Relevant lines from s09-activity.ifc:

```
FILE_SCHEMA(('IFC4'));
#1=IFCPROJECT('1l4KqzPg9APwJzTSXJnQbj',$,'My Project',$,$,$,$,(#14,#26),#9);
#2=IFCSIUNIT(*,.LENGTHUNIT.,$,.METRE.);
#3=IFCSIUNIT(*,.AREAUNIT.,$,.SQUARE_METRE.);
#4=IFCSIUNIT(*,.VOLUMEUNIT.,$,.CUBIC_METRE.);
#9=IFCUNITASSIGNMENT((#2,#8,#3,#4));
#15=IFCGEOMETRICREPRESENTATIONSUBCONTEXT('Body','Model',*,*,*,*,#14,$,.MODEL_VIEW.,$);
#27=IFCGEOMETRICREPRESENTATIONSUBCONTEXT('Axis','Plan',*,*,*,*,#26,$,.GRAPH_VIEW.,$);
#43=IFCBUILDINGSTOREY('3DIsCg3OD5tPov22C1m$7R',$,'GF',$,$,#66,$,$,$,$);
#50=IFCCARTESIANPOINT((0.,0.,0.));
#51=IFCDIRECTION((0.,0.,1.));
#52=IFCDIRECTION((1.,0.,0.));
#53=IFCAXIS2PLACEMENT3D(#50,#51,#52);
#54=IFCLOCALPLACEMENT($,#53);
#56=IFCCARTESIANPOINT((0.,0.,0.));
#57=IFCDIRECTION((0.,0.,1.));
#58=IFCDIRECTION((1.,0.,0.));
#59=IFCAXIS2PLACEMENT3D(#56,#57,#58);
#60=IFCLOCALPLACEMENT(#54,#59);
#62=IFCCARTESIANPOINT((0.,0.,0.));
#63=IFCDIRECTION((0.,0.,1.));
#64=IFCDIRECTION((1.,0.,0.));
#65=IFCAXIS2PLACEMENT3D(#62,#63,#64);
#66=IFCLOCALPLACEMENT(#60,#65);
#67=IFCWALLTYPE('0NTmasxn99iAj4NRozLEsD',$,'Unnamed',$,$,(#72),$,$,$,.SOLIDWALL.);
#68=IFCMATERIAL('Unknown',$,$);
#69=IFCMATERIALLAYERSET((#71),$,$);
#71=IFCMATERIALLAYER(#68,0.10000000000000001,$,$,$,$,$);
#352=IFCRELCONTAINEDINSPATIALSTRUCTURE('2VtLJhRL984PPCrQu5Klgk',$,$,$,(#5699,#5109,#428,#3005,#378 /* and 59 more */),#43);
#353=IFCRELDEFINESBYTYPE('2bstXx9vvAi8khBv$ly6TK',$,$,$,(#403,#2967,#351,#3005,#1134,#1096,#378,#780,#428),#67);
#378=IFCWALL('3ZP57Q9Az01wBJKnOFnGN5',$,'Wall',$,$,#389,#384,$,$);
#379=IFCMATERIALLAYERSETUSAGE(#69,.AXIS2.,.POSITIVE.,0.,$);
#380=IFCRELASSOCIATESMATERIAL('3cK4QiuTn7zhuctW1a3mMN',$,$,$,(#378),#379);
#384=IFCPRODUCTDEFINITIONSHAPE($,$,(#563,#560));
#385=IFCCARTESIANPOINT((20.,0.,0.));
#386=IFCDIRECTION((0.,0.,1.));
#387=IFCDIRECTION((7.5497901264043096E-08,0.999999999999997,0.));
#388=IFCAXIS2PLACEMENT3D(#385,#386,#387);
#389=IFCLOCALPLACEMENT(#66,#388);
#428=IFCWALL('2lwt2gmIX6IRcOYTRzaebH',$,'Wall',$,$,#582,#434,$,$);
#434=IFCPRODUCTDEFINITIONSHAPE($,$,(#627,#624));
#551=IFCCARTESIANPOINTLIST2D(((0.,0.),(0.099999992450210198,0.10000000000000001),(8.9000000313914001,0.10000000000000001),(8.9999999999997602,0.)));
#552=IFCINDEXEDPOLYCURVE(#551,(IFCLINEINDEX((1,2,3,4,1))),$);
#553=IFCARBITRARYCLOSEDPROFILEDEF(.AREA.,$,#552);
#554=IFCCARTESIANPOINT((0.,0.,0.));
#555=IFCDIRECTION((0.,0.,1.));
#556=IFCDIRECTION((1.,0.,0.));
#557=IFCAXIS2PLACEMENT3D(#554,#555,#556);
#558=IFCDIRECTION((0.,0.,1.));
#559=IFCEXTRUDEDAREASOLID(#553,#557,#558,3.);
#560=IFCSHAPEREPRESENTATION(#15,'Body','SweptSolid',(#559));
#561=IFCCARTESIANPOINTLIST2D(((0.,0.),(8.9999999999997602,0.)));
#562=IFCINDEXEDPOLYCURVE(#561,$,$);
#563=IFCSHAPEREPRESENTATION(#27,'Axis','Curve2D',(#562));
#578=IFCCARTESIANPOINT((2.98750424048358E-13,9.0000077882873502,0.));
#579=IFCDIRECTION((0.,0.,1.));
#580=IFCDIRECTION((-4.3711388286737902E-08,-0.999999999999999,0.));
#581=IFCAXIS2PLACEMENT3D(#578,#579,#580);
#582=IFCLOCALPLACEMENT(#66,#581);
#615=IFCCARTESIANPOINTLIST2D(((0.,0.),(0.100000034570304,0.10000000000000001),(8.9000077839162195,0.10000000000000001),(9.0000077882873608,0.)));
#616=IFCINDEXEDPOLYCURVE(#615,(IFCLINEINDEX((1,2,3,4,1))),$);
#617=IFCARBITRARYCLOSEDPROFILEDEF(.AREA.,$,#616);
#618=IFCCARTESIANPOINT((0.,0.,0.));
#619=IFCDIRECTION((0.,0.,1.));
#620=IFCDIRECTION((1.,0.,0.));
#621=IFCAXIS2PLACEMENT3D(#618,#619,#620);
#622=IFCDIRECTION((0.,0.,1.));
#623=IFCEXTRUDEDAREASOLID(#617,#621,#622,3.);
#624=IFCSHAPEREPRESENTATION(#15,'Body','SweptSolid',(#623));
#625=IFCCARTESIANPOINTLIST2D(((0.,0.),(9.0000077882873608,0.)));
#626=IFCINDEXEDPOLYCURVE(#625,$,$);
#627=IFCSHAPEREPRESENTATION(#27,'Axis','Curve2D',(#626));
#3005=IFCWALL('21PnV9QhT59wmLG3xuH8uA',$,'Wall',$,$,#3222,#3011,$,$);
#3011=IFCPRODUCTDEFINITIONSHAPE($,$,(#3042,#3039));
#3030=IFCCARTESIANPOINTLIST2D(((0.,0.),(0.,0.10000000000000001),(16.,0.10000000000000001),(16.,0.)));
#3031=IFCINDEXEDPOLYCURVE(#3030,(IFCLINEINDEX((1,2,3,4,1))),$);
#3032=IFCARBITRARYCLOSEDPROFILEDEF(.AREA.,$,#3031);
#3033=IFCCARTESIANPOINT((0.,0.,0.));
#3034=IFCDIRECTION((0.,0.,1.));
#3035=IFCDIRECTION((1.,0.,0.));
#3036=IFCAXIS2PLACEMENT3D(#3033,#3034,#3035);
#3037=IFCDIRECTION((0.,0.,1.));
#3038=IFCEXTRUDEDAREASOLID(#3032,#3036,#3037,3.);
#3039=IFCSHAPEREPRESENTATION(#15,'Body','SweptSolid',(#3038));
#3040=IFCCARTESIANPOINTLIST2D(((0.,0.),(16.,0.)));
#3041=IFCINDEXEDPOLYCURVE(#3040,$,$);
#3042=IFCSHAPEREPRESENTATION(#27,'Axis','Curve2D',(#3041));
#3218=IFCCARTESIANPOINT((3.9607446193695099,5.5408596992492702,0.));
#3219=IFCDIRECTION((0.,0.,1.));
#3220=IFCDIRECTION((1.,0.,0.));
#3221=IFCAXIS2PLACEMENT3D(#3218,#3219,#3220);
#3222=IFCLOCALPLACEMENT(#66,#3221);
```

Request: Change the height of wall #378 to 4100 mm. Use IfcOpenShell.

```python
import ifcopenshell
import ifcopenshell.geom
import ifcopenshell.util.representation
import ifcopenshell.util.shape
import ifcopenshell.util.unit

model = ifcopenshell.open("s09-activity.ifc")
unit_scale = ifcopenshell.util.unit.calculate_unit_scale(model)
settings = ifcopenshell.geom.settings()


def volume(element):
    """Net volume in cubic metres, openings subtracted."""
    shape = ifcopenshell.geom.create_shape(settings, element)
    return ifcopenshell.util.shape.get_volume(shape.geometry)


wall = model.by_id(378)
before = volume(wall)

body = ifcopenshell.util.representation.get_representation(wall, "Model", "Body")
solid = body.Items[0]
old_height = solid.Depth
solid.Depth = 4.1 / unit_scale
after = volume(wall)

print(f"height {old_height:g} -> {solid.Depth:g}, volume {before:.3f} -> {after:.3f} m3")

model.write("s09-activity_edited.ifc")
```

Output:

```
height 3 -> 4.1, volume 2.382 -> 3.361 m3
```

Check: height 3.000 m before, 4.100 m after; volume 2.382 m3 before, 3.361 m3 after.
